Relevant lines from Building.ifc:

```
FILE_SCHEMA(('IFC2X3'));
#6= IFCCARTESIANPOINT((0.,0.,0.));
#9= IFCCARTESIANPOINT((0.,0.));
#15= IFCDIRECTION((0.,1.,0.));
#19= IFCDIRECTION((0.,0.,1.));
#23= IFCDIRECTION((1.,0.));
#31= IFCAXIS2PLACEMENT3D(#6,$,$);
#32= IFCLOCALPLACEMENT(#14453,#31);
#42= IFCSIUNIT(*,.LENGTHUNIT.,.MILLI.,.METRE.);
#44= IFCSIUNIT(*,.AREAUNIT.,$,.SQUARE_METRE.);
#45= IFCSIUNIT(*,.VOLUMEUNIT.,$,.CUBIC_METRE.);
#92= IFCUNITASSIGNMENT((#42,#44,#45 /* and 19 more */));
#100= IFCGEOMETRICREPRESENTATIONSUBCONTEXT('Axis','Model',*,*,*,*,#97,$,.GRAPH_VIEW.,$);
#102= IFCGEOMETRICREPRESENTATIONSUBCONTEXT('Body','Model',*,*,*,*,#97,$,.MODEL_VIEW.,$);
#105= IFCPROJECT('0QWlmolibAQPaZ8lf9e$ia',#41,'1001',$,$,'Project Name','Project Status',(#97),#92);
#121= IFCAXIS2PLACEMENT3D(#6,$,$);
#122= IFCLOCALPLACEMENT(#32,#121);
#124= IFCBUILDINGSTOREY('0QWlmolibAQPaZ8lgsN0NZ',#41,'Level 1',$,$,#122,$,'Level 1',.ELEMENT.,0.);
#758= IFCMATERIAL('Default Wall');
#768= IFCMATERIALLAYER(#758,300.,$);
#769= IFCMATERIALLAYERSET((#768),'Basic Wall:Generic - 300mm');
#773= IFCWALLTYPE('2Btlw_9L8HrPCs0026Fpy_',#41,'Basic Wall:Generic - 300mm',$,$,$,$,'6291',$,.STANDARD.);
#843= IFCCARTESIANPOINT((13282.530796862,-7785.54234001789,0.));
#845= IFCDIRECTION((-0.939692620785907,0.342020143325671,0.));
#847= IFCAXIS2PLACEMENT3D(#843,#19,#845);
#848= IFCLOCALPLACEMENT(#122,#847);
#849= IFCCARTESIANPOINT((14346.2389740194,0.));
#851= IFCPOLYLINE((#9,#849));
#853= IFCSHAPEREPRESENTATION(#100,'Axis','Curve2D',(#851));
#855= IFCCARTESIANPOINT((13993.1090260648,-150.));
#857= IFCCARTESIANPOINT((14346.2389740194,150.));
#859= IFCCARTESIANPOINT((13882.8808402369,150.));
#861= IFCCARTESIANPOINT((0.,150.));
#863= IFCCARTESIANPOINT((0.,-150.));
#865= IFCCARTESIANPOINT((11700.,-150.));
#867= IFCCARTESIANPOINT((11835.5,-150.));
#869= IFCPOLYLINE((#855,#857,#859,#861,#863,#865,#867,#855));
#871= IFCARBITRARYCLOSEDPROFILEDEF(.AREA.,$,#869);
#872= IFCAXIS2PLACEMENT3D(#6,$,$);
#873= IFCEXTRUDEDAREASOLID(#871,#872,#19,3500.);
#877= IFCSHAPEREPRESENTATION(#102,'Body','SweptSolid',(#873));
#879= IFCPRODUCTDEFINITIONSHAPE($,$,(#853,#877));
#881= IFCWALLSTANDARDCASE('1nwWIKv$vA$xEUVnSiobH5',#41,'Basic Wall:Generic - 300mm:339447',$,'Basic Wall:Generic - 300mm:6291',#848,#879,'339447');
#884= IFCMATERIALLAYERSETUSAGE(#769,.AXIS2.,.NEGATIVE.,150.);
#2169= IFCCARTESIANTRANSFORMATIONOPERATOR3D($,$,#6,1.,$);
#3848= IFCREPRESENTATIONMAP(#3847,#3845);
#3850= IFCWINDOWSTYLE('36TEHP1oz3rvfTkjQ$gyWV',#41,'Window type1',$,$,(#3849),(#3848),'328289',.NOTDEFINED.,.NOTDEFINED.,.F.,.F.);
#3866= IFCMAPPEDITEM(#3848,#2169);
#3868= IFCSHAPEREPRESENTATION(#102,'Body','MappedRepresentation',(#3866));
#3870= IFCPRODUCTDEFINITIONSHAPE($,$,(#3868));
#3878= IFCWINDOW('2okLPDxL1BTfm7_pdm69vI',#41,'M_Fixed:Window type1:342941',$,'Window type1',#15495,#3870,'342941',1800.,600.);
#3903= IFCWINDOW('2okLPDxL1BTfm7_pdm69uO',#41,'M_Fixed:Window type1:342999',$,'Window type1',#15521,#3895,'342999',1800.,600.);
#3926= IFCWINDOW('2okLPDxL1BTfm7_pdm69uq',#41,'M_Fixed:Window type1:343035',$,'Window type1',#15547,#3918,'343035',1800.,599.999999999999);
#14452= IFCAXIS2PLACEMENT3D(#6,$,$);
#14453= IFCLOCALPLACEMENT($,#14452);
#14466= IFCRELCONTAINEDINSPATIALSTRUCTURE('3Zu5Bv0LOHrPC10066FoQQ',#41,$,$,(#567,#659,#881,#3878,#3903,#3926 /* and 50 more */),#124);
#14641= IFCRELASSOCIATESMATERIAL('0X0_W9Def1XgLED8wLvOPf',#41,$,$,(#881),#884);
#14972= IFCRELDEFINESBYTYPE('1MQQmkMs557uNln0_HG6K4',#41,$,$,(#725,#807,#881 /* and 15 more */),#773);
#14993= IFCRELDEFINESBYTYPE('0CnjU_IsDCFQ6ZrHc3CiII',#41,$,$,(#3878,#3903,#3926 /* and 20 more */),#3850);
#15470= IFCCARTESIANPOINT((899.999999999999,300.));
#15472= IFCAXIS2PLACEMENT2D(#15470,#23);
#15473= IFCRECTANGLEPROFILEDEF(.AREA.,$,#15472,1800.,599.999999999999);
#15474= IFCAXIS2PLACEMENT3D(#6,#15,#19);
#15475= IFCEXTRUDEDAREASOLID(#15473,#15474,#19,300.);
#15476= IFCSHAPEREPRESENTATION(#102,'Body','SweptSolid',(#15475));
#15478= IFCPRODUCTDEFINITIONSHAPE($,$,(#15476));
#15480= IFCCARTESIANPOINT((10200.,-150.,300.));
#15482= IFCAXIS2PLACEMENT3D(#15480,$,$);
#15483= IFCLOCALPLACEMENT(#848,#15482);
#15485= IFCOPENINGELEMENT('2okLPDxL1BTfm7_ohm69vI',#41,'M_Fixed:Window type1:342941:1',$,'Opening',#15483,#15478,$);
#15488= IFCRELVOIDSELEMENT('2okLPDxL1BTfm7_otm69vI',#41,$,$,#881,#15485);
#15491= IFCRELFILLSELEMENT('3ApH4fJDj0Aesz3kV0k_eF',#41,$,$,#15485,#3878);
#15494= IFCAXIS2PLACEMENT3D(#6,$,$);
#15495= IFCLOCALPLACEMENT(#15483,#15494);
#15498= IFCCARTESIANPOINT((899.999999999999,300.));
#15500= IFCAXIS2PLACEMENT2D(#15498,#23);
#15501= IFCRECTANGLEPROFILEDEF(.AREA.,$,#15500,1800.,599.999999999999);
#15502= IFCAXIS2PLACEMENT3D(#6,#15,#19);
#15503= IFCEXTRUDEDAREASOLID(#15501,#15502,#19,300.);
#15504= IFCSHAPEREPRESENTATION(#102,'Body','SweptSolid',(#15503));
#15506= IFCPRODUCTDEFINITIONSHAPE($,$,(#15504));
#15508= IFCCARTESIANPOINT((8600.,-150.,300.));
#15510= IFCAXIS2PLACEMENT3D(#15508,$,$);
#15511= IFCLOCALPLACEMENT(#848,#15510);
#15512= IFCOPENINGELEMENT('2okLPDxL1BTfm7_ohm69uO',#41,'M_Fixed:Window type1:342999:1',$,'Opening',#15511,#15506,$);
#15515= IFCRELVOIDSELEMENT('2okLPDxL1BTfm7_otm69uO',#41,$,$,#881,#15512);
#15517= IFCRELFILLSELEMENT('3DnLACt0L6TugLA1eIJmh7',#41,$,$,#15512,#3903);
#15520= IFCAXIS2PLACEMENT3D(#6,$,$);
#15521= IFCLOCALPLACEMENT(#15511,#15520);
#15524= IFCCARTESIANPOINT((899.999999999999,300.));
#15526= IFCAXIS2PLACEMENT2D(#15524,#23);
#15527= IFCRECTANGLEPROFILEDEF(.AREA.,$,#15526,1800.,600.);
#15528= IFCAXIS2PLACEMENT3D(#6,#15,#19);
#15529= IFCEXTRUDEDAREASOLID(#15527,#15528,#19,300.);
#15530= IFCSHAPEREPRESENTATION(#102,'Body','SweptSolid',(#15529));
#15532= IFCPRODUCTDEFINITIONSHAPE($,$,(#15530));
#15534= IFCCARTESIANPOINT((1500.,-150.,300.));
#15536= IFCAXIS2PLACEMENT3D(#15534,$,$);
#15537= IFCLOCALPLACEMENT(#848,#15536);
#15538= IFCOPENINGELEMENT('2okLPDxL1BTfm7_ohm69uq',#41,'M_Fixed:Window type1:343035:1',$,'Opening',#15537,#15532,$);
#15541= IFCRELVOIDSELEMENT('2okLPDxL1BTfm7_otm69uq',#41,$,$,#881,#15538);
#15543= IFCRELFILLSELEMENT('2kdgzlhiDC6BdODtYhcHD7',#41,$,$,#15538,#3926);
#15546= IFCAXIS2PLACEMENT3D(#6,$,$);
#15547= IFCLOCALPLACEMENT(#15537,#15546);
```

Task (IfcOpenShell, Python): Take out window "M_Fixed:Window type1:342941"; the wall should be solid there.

```python
import ifcopenshell
import ifcopenshell.api.feature
import ifcopenshell.api.root
import ifcopenshell.geom
import ifcopenshell.util.shape

model = ifcopenshell.open("Building.ifc")
settings = ifcopenshell.geom.settings()


def volume(element):
    """Net volume in cubic metres, openings subtracted."""
    shape = ifcopenshell.geom.create_shape(settings, element)
    return ifcopenshell.util.shape.get_volume(shape.geometry)


window = model.by_guid("2okLPDxL1BTfm7_pdm69vI")
opening = window.FillsVoids[0].RelatingOpeningElement
wall = opening.VoidsElements[0].RelatingBuildingElement
before = volume(wall)

ifcopenshell.api.root.remove_product(model, product=window)
ifcopenshell.api.feature.remove_feature(model, feature=opening)

after = volume(wall)

print(f"wall volume {before:.3f} -> {after:.3f} m3")

model.write("Building-out.ifc")
```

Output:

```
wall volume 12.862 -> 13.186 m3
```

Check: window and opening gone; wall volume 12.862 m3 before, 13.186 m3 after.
